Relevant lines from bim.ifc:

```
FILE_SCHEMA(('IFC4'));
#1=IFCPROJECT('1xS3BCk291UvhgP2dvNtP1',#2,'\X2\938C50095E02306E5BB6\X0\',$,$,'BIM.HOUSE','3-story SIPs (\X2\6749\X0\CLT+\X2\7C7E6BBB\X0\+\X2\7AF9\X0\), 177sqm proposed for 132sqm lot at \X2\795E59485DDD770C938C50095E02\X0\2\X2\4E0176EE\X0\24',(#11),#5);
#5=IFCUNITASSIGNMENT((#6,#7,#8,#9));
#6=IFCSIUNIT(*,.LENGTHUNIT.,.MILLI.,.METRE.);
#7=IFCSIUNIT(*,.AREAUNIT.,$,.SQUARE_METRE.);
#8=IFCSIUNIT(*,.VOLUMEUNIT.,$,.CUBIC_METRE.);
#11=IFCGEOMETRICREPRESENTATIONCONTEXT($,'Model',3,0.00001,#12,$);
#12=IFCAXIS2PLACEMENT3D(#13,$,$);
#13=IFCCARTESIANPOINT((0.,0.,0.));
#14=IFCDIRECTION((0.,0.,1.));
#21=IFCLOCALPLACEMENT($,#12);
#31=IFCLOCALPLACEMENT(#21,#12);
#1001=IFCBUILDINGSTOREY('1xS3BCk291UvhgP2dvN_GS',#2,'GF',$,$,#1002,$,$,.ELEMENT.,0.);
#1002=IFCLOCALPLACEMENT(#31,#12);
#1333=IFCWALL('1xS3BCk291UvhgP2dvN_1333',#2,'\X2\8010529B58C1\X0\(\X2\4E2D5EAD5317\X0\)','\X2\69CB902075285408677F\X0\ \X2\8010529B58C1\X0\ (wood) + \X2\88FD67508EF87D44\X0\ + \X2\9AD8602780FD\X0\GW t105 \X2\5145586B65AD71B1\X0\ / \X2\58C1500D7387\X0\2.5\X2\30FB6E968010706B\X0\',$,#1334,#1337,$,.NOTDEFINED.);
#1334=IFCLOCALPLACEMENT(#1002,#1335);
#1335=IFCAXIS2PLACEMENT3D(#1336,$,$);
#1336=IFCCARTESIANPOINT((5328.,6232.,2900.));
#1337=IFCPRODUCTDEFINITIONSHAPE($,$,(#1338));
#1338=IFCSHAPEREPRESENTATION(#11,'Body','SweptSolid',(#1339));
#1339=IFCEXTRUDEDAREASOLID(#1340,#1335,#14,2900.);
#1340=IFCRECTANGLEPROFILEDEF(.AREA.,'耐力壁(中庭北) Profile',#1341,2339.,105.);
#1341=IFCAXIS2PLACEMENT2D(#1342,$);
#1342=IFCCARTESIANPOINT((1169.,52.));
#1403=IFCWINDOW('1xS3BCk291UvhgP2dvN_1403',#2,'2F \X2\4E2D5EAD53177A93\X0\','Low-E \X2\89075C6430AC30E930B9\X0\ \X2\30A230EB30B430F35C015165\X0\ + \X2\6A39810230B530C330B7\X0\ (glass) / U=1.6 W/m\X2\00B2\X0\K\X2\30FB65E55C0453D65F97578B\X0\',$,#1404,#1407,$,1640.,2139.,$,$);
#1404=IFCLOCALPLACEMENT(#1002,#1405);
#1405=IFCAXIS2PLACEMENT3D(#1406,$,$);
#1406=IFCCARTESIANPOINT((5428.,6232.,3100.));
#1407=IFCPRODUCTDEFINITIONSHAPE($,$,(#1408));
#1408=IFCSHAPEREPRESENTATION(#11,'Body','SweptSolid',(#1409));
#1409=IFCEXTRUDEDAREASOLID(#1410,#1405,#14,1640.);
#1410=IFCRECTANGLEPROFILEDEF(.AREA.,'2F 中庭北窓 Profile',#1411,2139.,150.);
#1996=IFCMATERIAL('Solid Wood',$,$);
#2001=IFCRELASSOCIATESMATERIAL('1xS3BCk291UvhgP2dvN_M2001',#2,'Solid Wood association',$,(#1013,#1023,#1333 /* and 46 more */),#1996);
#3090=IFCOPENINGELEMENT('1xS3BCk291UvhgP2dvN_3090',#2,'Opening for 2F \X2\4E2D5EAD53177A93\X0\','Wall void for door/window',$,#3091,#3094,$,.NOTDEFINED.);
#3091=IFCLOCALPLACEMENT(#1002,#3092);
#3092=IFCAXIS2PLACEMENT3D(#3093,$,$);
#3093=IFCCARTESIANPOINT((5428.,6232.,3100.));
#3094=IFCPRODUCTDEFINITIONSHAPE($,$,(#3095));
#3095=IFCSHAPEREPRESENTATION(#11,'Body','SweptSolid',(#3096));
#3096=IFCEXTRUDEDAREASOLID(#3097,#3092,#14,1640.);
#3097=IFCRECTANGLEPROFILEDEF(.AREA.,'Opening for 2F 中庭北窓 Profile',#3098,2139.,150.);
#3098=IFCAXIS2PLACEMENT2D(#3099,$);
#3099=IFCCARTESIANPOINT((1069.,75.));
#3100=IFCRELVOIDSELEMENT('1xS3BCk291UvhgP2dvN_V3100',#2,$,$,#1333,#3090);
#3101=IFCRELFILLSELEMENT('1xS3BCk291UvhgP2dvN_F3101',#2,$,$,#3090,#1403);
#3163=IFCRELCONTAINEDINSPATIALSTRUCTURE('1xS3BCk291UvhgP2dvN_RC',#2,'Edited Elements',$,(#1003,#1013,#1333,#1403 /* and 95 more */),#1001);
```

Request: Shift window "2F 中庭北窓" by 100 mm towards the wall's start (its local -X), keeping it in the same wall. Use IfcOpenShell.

```python
import ifcopenshell
import ifcopenshell.api.geometry
import ifcopenshell.util.placement
import ifcopenshell.util.unit

model = ifcopenshell.open("bim.ifc")
unit_scale = ifcopenshell.util.unit.calculate_unit_scale(model)

window = model.by_id(1403)
opening = window.FillsVoids[0].RelatingOpeningElement
wall = opening.VoidsElements[0].RelatingBuildingElement

wall_matrix = ifcopenshell.util.placement.get_local_placement(wall.ObjectPlacement)
shift = wall_matrix[:3, 0] * -0.1 / unit_scale
before = ifcopenshell.util.placement.get_local_placement(window.ObjectPlacement)[:3, 3].copy()

# The window is not placed relative to its opening, so move both.
for product in (opening, window):
    matrix = ifcopenshell.util.placement.get_local_placement(product.ObjectPlacement)
    matrix[:3, 3] += shift
    ifcopenshell.api.geometry.edit_object_placement(model, product=product, matrix=matrix, is_si=False)

after = ifcopenshell.util.placement.get_local_placement(window.ObjectPlacement)[:3, 3]
print("window moved by", (after - before).round(3) + 0.0)

model.write("bim-out.ifc")
```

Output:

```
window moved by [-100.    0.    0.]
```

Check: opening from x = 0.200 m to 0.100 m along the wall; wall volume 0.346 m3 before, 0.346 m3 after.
